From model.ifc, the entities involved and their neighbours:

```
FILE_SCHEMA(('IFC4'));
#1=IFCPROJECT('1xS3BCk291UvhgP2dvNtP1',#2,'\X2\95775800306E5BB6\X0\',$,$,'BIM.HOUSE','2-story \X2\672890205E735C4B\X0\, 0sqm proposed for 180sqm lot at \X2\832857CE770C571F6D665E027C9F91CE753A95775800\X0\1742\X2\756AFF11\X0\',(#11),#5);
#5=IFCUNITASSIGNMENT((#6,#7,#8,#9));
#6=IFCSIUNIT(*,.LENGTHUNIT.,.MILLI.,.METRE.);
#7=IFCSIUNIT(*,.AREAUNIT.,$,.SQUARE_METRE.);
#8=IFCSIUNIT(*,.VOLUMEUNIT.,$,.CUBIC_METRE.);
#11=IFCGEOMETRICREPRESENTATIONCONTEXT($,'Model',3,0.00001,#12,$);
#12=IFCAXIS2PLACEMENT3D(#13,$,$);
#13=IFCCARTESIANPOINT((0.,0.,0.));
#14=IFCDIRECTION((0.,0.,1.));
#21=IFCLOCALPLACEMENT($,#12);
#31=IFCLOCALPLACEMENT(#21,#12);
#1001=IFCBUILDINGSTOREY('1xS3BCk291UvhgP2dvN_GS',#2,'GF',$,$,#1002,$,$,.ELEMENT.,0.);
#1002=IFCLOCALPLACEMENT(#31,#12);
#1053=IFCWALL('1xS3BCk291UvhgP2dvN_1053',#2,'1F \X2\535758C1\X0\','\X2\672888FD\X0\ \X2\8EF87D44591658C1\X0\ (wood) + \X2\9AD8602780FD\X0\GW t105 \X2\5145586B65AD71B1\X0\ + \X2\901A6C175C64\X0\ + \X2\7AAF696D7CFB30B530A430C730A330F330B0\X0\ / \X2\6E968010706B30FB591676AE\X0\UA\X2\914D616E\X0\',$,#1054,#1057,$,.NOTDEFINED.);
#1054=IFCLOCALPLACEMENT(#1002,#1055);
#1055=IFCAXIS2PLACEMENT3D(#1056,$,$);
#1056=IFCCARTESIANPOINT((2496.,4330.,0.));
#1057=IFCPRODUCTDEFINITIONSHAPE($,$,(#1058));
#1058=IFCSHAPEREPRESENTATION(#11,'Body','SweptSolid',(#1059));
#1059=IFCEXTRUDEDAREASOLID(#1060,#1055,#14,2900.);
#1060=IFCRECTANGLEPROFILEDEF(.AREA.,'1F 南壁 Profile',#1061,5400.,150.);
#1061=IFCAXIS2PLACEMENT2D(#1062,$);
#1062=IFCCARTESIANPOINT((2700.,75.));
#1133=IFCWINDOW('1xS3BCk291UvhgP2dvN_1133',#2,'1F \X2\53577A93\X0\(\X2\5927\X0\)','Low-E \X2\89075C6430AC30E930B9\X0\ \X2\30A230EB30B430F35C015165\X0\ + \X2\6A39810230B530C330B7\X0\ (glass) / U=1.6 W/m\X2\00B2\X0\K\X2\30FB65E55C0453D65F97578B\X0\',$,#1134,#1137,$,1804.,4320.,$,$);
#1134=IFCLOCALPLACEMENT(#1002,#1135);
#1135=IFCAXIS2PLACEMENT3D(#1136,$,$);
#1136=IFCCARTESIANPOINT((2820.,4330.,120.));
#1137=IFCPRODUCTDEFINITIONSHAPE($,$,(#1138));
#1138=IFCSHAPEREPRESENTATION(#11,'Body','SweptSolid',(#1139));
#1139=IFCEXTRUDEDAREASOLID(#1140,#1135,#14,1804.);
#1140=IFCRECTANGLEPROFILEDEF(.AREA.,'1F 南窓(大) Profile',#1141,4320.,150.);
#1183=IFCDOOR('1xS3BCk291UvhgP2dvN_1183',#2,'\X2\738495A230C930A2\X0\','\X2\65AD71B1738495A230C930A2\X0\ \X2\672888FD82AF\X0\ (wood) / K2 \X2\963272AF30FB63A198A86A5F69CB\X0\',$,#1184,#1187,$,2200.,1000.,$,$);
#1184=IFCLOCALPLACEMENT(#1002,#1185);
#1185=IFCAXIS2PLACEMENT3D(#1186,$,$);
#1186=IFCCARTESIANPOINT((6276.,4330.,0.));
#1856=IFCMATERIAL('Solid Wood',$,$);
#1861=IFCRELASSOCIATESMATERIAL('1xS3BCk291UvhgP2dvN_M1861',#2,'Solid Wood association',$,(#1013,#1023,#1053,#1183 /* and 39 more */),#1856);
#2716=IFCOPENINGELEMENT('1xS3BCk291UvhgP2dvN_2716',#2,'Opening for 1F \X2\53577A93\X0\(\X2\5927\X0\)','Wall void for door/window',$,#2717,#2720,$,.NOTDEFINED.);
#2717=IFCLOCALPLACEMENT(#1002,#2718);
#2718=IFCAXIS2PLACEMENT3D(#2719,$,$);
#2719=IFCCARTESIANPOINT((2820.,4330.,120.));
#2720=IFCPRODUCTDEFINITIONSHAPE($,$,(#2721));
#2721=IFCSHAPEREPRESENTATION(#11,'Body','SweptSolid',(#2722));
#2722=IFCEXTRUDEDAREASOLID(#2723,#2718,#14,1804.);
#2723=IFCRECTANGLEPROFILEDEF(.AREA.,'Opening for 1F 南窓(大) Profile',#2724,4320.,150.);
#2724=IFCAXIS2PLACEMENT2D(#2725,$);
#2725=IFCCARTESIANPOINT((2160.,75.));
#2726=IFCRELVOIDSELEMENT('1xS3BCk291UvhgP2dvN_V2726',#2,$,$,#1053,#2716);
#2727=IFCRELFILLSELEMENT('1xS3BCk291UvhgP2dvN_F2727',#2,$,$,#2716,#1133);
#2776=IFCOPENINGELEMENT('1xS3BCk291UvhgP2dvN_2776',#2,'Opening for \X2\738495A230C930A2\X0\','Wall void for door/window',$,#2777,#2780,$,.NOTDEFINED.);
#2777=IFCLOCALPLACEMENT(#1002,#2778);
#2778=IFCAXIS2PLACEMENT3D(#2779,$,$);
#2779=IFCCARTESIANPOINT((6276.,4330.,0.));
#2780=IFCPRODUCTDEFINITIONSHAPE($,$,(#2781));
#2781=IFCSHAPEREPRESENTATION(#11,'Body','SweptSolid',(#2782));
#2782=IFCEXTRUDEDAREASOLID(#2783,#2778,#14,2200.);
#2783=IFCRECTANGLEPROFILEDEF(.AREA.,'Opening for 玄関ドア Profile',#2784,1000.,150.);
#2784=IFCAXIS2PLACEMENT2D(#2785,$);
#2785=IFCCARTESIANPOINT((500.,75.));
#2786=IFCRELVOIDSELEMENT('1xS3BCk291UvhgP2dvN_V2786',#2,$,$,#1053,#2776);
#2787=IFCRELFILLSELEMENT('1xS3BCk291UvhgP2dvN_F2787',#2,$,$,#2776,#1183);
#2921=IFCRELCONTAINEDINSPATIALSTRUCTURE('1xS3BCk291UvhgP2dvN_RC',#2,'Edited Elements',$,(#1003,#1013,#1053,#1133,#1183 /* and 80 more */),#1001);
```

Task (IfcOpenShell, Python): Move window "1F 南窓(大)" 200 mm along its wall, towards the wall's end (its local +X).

```python
import ifcopenshell
import ifcopenshell.api.geometry
import ifcopenshell.util.placement
import ifcopenshell.util.unit

model = ifcopenshell.open("model.ifc")
unit_scale = ifcopenshell.util.unit.calculate_unit_scale(model)

window = model.by_guid("1xS3BCk291UvhgP2dvN_1133")
opening = window.FillsVoids[0].RelatingOpeningElement
wall = opening.VoidsElements[0].RelatingBuildingElement

wall_matrix = ifcopenshell.util.placement.get_local_placement(wall.ObjectPlacement)
shift = wall_matrix[:3, 0] * 0.2 / unit_scale
before = ifcopenshell.util.placement.get_local_placement(window.ObjectPlacement)[:3, 3].copy()

# The window is not placed relative to its opening, so move both.
for product in (opening, window):
    matrix = ifcopenshell.util.placement.get_local_placement(product.ObjectPlacement)
    matrix[:3, 3] += shift
    ifcopenshell.api.geometry.edit_object_placement(model, product=product, matrix=matrix, is_si=False)

after = ifcopenshell.util.placement.get_local_placement(window.ObjectPlacement)[:3, 3]
print("window moved by", (after - before).round(3) + 0.0)

model.write("model_edited.ifc")
```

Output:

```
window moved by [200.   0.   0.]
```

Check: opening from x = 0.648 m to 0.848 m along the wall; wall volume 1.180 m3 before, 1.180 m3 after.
